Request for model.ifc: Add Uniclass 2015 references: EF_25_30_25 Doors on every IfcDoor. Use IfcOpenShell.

First a look at what the model holds.

```python
import ifcopenshell

model = ifcopenshell.open("model.ifc")
print(model.schema)
print("classifications:", [c.Name for c in model.by_type("IfcClassification")])
for ifc_class in ("IfcDoor", "IfcRoof", "IfcStair", "IfcWall", "IfcWindow"):
    print(ifc_class, len(model.by_type(ifc_class)))
```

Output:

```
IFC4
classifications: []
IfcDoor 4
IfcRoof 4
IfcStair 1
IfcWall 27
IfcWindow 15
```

```python
import ifcopenshell
import ifcopenshell.api.classification

model = ifcopenshell.open("model.ifc")

system = ifcopenshell.api.classification.add_classification(model, classification="Uniclass 2015")

codes = {
    "IfcDoor": ("EF_25_30_25", "Doors"),
}
for ifc_class, (code, name) in codes.items():
    products = model.by_type(ifc_class)
    ifcopenshell.api.classification.add_reference(
        model, products=products, classification=system, identification=code, name=name
    )
    print(code, len(products))

model.write("model_edited.ifc")
```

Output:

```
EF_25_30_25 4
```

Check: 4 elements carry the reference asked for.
